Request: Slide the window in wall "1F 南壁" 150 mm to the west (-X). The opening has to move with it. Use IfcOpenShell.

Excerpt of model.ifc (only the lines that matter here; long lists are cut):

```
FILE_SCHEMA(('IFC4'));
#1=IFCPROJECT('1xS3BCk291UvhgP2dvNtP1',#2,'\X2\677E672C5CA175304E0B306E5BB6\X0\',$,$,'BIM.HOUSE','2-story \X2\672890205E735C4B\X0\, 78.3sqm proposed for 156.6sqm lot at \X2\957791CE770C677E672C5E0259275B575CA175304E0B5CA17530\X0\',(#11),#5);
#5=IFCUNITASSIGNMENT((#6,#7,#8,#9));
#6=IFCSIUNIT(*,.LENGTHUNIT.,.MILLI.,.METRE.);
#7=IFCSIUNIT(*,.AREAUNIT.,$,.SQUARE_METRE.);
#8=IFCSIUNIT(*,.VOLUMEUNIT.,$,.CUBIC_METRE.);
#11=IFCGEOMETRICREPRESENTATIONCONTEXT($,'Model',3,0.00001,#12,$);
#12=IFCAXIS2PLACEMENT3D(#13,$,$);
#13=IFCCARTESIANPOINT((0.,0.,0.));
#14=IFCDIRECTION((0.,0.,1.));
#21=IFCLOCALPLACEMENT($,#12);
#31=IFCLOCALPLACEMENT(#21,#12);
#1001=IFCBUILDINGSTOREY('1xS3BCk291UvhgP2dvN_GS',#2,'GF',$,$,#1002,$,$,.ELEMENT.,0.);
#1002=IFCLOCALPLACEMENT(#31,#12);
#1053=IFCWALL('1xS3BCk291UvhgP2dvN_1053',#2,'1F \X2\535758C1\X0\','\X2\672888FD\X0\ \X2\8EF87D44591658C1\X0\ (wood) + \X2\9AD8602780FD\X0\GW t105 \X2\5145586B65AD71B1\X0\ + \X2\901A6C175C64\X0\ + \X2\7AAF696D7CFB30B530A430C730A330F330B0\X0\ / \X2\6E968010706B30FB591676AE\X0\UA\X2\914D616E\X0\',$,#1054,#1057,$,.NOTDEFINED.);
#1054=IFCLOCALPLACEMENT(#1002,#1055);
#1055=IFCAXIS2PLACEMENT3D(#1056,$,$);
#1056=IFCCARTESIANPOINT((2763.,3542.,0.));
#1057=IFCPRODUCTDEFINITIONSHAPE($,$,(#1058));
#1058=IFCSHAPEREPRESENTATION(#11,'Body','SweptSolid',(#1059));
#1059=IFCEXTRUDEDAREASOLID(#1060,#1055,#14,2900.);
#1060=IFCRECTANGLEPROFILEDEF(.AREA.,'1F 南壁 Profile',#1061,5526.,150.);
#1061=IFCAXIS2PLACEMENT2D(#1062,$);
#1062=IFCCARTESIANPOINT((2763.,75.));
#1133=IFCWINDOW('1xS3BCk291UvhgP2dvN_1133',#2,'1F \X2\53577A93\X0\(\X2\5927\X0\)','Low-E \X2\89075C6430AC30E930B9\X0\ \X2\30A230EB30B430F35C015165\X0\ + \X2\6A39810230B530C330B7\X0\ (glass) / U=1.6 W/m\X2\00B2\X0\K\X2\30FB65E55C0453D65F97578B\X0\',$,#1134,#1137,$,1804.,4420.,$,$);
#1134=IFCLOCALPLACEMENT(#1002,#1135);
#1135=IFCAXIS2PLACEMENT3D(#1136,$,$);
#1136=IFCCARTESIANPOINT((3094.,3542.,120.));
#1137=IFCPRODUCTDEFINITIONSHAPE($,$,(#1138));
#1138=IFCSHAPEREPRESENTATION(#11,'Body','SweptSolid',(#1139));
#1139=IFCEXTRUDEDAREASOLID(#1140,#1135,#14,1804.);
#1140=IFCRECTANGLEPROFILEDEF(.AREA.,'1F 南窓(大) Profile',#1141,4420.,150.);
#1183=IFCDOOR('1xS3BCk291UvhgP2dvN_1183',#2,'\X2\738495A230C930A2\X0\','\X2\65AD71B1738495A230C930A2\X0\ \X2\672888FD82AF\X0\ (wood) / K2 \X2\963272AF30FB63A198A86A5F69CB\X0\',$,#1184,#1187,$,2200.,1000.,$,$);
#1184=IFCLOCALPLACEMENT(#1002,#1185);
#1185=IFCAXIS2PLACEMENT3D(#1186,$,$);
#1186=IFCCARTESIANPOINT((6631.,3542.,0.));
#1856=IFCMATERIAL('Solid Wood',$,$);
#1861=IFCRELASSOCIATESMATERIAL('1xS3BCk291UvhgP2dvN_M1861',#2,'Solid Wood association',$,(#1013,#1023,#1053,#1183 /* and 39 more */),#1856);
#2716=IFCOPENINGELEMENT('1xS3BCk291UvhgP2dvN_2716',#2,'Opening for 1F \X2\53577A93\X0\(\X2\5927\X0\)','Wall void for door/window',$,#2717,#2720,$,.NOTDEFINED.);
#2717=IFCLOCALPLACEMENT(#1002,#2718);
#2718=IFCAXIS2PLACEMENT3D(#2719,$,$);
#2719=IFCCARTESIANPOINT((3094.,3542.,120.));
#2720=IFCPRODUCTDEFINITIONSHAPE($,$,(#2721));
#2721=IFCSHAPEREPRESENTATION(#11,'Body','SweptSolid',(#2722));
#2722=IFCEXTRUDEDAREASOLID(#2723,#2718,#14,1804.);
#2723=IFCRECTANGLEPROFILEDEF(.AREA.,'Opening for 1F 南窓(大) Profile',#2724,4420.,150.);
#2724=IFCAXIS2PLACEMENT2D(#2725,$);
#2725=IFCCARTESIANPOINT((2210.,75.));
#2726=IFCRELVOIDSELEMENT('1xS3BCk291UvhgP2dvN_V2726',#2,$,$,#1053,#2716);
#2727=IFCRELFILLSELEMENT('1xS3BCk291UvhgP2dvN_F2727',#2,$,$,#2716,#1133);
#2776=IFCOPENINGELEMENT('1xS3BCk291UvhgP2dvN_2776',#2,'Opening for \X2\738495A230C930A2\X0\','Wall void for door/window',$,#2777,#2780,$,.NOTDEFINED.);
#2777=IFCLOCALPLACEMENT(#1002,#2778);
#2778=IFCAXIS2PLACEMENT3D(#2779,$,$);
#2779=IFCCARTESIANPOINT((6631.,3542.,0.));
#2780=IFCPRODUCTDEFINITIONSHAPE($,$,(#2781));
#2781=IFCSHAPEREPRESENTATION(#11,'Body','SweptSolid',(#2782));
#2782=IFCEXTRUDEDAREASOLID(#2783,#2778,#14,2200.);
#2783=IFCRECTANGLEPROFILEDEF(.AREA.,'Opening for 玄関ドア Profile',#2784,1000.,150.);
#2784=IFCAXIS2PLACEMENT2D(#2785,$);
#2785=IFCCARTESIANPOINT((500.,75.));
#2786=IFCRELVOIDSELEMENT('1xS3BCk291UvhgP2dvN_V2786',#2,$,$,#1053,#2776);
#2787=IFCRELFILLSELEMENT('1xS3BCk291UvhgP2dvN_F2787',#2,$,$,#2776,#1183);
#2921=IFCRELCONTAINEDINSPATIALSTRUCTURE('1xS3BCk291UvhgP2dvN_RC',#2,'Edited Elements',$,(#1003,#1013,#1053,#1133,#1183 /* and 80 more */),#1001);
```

```python
import ifcopenshell
import ifcopenshell.api.geometry
import ifcopenshell.util.placement

model = ifcopenshell.open("model.ifc")

window = model.by_id(1133)
opening = window.FillsVoids[0].RelatingOpeningElement
wall = opening.VoidsElements[0].RelatingBuildingElement

wall_matrix = ifcopenshell.util.placement.get_local_placement(wall.ObjectPlacement)
shift = wall_matrix[:3, 0] * -150.0
before = ifcopenshell.util.placement.get_local_placement(window.ObjectPlacement)[:3, 3].copy()

# The window is not placed relative to its opening, so move both.
for product in (opening, window):
    matrix = ifcopenshell.util.placement.get_local_placement(product.ObjectPlacement)
    matrix[:3, 3] += shift
    ifcopenshell.api.geometry.edit_object_placement(model, product=product, matrix=matrix, is_si=False)

after = ifcopenshell.util.placement.get_local_placement(window.ObjectPlacement)[:3, 3]
print("window moved by", (after - before).round(3) + 0.0)

model.write("model_rev.ifc")
```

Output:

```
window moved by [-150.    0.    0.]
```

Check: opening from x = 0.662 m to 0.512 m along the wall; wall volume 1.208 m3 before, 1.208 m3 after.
